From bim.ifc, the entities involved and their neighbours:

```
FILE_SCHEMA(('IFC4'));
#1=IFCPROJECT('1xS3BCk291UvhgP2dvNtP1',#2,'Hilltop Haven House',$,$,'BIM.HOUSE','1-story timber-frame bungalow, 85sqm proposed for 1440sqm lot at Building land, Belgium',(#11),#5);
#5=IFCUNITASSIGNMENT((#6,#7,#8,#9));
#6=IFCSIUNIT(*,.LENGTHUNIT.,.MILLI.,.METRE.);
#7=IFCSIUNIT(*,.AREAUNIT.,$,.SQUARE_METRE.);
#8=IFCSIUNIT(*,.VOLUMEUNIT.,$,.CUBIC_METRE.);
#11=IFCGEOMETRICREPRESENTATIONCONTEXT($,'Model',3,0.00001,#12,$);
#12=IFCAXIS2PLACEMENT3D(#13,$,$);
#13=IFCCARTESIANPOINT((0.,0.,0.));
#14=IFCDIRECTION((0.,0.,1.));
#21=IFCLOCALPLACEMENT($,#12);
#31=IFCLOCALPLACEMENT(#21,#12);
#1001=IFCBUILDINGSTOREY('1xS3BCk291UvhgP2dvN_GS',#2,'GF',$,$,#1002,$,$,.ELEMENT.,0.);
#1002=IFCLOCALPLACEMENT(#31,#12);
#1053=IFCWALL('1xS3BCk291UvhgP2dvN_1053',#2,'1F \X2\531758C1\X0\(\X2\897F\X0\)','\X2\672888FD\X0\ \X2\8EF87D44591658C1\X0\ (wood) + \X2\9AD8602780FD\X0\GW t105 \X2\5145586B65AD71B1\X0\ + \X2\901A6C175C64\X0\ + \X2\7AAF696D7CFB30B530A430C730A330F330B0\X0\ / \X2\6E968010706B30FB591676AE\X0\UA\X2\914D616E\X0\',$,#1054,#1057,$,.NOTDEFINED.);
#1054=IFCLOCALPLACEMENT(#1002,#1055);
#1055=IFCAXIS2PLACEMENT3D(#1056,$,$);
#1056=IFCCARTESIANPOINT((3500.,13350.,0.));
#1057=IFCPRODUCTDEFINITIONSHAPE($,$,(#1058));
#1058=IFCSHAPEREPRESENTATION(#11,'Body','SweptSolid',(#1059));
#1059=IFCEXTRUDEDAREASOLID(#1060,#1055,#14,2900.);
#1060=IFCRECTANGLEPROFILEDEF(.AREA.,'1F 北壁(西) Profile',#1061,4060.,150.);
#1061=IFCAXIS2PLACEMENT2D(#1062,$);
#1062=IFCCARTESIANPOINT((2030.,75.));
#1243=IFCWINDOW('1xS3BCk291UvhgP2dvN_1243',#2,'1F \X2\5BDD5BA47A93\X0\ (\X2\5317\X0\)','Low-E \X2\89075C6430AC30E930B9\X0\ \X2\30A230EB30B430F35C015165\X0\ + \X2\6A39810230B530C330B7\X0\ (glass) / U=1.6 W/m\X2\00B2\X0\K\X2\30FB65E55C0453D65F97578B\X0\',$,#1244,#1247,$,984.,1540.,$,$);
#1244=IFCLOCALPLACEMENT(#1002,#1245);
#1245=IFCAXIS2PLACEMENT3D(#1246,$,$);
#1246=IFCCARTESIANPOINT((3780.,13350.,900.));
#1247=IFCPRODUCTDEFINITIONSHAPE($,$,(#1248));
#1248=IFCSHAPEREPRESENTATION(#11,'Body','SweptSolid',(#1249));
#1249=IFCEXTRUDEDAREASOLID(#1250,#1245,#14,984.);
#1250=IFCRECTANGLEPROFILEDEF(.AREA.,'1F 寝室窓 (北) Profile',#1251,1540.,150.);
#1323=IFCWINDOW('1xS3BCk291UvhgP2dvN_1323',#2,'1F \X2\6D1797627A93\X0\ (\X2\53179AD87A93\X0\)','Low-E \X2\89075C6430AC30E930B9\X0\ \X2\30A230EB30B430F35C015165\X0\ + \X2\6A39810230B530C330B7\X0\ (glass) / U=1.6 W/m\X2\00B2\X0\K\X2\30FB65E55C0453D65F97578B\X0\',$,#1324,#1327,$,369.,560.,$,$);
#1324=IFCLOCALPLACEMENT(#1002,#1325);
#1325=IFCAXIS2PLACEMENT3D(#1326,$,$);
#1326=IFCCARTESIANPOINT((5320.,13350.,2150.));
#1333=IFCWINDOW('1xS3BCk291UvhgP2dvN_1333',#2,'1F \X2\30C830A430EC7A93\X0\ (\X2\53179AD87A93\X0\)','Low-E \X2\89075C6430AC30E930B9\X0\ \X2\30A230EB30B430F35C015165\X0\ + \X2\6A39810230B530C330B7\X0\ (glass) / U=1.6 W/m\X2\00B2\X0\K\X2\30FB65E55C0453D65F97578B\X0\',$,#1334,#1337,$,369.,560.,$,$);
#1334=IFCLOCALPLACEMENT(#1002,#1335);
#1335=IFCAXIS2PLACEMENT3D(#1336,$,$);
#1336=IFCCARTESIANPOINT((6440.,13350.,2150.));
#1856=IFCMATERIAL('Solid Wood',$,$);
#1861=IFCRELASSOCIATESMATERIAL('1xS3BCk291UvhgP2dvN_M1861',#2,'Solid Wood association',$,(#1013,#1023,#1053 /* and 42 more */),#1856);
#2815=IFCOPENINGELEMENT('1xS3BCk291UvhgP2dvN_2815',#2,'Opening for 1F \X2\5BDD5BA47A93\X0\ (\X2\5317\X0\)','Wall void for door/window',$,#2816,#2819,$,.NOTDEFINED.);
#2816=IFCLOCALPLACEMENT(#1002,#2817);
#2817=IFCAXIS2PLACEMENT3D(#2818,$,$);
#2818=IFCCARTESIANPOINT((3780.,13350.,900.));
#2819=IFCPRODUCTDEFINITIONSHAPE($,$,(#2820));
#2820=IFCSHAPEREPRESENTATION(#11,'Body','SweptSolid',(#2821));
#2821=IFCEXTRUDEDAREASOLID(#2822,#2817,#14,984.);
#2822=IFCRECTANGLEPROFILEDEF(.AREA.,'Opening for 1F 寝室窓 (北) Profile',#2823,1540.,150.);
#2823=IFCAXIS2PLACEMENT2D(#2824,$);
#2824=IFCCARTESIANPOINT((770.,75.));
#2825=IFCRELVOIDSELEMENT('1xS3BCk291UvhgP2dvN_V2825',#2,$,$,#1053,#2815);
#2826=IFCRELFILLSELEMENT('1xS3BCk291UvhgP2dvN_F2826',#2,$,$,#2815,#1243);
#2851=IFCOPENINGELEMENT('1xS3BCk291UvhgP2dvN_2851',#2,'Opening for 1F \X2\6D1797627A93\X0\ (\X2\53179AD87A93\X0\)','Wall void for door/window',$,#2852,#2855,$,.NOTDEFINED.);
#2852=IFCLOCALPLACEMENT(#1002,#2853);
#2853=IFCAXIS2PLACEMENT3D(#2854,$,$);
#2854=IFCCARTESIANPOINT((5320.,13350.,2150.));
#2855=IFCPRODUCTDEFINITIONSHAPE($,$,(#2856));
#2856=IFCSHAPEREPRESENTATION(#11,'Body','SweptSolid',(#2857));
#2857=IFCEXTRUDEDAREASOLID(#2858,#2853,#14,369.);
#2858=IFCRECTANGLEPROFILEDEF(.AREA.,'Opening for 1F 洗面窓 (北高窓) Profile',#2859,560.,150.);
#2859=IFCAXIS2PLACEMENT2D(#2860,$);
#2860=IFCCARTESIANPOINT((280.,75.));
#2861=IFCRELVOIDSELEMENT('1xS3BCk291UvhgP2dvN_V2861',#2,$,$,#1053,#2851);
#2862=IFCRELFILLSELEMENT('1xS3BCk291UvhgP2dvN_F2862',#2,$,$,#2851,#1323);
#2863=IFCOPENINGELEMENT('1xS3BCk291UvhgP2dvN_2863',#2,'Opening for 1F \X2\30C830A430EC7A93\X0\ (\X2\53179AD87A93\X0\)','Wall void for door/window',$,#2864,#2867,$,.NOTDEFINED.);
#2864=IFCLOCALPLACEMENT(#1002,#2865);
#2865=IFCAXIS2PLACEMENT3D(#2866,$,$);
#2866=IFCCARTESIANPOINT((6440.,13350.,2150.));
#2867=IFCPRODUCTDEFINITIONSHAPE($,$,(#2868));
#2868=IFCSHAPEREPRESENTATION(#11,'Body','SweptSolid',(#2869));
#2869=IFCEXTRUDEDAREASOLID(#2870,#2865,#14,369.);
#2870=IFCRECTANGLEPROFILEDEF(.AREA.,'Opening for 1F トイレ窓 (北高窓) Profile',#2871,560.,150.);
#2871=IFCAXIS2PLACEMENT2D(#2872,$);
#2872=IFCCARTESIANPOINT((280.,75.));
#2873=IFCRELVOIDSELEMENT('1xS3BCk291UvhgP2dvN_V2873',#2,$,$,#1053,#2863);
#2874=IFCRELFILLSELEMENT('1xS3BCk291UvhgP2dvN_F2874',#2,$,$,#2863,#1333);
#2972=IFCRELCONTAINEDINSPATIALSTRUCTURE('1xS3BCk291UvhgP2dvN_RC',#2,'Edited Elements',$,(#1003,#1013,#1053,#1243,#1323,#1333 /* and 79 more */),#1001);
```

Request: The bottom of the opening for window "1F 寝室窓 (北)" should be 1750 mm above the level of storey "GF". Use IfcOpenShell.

```python
import numpy as np
import ifcopenshell
import ifcopenshell.api.geometry
import ifcopenshell.geom
import ifcopenshell.util.element
import ifcopenshell.util.placement
import ifcopenshell.util.shape
import ifcopenshell.util.unit

model = ifcopenshell.open("bim.ifc")
unit_scale = ifcopenshell.util.unit.calculate_unit_scale(model)

window = model.by_guid("1xS3BCk291UvhgP2dvN_1243")
opening = window.FillsVoids[0].RelatingOpeningElement
storey = ifcopenshell.util.element.get_container(window, ifc_class="IfcBuildingStorey")
level = ifcopenshell.util.placement.get_local_placement(storey.ObjectPlacement)[2, 3]

# The opening's origin need not be at the sill, so measure its lowest point.
shape = ifcopenshell.geom.create_shape(ifcopenshell.geom.settings(), opening)
bottom = ifcopenshell.util.shape.get_shape_bottom_elevation(shape, shape.geometry) / unit_scale
dz = level + 1750.0 - bottom

shift = np.array([0.0, 0.0, dz])
# The window is not placed relative to its opening, so move both.
for product in (opening, window):
    matrix = ifcopenshell.util.placement.get_local_placement(product.ObjectPlacement)
    matrix[:3, 3] += shift
    ifcopenshell.api.geometry.edit_object_placement(model, product=product, matrix=matrix, is_si=False)

print(f"moved by {dz * unit_scale:+.3f} m")

model.write("bim_v2.ifc")
```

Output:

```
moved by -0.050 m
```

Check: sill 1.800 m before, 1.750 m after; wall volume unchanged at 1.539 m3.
